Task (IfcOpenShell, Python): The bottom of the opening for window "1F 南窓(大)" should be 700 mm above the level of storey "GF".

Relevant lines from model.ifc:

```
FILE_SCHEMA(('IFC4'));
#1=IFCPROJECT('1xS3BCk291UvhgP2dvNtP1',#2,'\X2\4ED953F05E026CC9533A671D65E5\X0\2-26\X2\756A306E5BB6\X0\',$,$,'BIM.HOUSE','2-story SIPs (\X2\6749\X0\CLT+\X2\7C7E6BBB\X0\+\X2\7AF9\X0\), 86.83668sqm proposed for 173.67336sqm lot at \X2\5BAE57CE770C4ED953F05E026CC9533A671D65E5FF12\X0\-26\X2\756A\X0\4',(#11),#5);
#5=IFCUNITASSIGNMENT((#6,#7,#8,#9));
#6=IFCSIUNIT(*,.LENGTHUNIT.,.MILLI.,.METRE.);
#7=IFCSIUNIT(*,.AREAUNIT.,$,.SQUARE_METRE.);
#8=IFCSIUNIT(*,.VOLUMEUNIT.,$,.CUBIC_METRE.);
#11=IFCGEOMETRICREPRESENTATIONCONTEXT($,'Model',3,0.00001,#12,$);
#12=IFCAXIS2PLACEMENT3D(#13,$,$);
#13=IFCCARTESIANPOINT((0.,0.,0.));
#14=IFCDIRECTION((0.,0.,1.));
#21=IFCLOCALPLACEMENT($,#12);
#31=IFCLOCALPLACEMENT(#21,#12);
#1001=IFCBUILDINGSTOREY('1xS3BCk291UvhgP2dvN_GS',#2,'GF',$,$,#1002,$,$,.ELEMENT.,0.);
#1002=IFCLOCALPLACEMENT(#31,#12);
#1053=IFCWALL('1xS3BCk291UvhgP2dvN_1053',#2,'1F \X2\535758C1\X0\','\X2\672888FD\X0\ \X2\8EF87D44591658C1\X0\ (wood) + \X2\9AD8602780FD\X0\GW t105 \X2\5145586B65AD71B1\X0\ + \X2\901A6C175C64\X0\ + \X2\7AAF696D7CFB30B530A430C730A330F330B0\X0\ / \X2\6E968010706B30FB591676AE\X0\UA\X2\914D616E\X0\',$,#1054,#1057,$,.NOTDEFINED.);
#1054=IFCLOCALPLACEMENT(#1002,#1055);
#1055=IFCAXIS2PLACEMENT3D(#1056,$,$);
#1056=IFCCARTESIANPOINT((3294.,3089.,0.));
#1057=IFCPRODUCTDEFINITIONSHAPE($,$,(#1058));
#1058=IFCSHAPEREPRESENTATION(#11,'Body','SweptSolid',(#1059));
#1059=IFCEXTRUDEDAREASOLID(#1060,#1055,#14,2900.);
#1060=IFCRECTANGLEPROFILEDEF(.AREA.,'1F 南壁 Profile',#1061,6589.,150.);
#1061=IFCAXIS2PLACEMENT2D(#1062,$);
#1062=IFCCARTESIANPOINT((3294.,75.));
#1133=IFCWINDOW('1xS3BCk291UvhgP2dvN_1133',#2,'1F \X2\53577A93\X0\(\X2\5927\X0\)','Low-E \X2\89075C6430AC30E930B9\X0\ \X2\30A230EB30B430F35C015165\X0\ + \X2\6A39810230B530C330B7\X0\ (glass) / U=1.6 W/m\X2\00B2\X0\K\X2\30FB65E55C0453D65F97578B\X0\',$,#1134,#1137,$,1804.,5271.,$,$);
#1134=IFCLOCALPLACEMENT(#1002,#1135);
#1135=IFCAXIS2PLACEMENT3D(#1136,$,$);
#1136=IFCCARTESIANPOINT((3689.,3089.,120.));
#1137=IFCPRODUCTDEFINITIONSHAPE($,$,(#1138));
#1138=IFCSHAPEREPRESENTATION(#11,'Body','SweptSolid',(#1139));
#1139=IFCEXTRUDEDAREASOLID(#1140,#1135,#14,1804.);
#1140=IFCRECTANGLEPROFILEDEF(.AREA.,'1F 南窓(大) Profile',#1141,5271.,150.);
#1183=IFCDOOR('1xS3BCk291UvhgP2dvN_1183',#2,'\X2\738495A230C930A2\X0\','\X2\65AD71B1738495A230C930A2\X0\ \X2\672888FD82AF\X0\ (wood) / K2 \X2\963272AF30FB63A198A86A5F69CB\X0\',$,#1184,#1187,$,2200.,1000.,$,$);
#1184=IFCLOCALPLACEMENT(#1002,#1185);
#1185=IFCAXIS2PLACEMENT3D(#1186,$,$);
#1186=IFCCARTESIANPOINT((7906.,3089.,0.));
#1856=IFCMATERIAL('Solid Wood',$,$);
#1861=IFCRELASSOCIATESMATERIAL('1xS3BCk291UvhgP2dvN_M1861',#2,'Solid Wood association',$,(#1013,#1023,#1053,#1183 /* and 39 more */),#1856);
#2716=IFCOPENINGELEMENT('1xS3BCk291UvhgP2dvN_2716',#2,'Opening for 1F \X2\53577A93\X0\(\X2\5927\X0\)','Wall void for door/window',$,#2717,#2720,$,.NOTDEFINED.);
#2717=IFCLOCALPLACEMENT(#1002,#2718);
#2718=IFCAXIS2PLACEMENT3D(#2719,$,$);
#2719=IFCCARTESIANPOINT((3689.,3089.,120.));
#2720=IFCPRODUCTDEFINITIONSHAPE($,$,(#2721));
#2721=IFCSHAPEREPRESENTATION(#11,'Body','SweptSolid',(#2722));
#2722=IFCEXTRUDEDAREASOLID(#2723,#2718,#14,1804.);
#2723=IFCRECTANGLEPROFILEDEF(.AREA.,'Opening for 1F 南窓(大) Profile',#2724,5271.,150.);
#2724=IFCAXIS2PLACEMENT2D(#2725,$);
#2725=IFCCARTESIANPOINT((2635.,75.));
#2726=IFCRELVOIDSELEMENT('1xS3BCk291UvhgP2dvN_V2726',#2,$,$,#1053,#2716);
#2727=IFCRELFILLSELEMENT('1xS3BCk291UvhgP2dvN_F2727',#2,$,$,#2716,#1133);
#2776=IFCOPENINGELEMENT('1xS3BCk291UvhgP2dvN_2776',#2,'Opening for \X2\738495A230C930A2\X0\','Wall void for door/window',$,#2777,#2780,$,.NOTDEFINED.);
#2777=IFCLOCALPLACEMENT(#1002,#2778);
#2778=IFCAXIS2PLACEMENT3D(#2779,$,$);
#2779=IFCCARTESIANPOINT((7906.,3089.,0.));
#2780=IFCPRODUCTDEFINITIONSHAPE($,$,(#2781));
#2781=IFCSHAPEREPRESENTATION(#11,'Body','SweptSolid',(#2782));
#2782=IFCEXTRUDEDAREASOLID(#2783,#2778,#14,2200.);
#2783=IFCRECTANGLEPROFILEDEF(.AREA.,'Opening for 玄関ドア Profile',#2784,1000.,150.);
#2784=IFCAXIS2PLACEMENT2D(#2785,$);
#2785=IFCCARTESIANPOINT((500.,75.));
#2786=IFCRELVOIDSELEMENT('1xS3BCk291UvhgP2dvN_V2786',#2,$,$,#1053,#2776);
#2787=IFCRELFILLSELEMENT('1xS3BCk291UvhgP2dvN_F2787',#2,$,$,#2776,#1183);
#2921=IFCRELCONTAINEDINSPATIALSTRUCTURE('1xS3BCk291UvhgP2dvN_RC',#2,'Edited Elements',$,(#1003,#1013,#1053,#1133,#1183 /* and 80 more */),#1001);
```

```python
import numpy as np
import ifcopenshell
import ifcopenshell.api.geometry
import ifcopenshell.geom
import ifcopenshell.util.element
import ifcopenshell.util.placement
import ifcopenshell.util.shape
import ifcopenshell.util.unit

model = ifcopenshell.open("model.ifc")
unit_scale = ifcopenshell.util.unit.calculate_unit_scale(model)

window = model.by_guid("1xS3BCk291UvhgP2dvN_1133")
opening = window.FillsVoids[0].RelatingOpeningElement
storey = ifcopenshell.util.element.get_container(window, ifc_class="IfcBuildingStorey")
level = ifcopenshell.util.placement.get_local_placement(storey.ObjectPlacement)[2, 3]

# The opening's origin need not be at the sill, so measure its lowest point.
shape = ifcopenshell.geom.create_shape(ifcopenshell.geom.settings(), opening)
bottom = ifcopenshell.util.shape.get_shape_bottom_elevation(shape, shape.geometry) / unit_scale
dz = level + 700.0 - bottom

shift = np.array([0.0, 0.0, dz])
# The window is not placed relative to its opening, so move both.
for product in (opening, window):
    matrix = ifcopenshell.util.placement.get_local_placement(product.ObjectPlacement)
    matrix[:3, 3] += shift
    ifcopenshell.api.geometry.edit_object_placement(model, product=product, matrix=matrix, is_si=False)

print(f"moved by {dz * unit_scale:+.3f} m")

model.write("model_updated.ifc")
```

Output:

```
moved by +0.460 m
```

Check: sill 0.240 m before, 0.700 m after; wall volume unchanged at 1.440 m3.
